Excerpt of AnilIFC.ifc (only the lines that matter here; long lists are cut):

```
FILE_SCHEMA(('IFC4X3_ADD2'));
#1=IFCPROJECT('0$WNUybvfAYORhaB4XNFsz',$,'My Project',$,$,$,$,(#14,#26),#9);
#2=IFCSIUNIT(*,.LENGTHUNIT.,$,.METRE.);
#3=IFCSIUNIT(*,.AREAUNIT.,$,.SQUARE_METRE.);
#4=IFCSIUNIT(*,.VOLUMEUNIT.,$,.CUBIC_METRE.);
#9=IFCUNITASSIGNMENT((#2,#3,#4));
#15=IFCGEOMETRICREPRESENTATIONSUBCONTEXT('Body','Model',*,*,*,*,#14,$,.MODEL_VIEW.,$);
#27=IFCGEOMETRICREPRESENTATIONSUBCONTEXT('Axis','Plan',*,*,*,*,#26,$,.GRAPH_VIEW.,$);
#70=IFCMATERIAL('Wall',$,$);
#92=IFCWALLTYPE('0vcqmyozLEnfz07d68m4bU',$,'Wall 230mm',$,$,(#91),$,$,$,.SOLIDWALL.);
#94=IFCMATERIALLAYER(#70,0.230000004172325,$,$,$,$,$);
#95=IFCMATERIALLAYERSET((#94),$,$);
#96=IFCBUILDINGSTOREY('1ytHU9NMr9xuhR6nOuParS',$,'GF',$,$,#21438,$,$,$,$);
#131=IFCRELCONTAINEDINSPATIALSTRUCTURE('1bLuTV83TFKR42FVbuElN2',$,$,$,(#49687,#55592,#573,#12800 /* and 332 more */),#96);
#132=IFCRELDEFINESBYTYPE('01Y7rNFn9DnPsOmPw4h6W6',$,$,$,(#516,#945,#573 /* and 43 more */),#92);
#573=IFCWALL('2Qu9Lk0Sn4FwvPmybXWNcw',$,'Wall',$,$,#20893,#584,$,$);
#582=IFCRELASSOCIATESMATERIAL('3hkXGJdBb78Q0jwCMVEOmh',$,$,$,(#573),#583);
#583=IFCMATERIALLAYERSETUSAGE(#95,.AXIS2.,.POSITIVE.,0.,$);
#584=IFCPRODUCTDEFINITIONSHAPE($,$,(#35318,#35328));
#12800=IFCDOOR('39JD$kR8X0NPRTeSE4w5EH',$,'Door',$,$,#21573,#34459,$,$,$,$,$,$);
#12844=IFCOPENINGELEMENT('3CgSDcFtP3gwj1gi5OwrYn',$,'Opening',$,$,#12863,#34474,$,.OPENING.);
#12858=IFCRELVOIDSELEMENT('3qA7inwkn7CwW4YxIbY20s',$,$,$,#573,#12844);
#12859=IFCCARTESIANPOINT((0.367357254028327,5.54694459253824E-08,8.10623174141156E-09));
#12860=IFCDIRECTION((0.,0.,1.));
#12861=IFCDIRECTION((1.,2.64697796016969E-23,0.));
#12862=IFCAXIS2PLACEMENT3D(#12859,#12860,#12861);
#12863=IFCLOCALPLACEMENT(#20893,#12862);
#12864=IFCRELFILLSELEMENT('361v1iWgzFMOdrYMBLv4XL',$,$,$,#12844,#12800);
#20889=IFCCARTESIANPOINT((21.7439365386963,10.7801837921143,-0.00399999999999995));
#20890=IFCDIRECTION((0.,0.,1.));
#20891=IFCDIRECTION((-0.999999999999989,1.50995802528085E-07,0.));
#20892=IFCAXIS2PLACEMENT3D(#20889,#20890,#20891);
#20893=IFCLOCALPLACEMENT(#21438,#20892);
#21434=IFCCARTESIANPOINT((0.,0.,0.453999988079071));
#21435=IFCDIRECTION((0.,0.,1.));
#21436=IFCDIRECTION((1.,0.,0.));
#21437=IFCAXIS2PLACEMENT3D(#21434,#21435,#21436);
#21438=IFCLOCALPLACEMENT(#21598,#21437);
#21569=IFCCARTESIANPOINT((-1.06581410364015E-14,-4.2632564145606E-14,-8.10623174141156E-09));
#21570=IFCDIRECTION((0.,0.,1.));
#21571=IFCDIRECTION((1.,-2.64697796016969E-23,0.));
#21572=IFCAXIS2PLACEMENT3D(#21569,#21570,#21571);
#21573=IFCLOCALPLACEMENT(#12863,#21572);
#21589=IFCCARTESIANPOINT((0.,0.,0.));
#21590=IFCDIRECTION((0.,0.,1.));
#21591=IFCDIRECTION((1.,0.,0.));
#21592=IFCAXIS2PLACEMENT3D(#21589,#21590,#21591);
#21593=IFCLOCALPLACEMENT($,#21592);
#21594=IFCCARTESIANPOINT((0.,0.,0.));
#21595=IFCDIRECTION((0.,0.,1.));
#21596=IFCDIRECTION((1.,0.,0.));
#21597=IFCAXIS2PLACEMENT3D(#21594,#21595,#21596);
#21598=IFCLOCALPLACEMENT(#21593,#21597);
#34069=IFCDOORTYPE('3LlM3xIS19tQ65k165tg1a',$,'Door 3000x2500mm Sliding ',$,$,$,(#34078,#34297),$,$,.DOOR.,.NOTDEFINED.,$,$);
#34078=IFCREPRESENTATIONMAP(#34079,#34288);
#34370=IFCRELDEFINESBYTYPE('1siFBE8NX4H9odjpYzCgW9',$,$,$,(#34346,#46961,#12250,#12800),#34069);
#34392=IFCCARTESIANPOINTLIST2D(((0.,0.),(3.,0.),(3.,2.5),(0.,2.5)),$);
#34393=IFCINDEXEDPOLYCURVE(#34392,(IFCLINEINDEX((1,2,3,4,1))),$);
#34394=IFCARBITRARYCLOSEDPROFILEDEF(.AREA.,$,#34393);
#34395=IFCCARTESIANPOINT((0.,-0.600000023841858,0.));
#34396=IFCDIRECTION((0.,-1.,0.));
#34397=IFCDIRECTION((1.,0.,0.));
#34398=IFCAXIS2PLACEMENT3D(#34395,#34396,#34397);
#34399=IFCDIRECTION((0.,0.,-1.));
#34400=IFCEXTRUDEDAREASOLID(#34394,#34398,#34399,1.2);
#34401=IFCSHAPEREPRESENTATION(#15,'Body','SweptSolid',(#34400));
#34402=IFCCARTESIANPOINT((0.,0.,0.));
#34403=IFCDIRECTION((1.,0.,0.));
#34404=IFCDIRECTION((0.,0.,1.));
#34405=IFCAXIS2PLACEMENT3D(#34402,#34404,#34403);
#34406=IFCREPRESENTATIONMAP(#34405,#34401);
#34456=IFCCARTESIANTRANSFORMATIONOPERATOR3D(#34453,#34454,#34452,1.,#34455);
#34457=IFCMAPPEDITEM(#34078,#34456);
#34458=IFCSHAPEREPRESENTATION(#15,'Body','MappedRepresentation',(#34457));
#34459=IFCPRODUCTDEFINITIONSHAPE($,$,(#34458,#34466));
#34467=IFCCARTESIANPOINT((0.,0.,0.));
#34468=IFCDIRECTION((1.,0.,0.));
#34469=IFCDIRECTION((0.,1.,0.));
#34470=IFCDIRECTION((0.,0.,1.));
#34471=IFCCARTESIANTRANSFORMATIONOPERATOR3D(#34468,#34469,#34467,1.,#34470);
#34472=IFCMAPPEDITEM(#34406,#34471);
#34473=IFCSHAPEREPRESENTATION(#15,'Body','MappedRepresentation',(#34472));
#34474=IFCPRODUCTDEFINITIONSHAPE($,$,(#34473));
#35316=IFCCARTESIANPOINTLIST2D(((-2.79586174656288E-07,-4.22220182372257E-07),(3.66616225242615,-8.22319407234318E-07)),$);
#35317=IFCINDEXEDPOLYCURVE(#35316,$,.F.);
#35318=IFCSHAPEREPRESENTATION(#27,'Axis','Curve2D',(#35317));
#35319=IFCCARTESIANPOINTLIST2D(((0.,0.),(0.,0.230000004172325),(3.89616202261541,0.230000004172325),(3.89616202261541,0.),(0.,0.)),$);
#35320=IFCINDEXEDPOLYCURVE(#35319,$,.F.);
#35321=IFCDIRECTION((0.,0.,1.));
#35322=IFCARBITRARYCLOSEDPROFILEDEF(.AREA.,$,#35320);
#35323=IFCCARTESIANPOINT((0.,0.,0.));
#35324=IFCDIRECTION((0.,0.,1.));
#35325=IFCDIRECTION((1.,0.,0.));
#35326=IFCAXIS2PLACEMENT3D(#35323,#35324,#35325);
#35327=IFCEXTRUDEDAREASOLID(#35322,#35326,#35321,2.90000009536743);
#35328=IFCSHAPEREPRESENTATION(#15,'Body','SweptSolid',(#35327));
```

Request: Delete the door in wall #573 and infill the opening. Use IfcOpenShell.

```python
import ifcopenshell
import ifcopenshell.api.feature
import ifcopenshell.api.root
import ifcopenshell.geom
import ifcopenshell.util.shape

model = ifcopenshell.open("AnilIFC.ifc")
settings = ifcopenshell.geom.settings()


def volume(element):
    """Net volume in cubic metres, openings subtracted."""
    shape = ifcopenshell.geom.create_shape(settings, element)
    return ifcopenshell.util.shape.get_volume(shape.geometry)


door = model.by_guid("39JD$kR8X0NPRTeSE4w5EH")
opening = door.FillsVoids[0].RelatingOpeningElement
wall = opening.VoidsElements[0].RelatingBuildingElement
before = volume(wall)

ifcopenshell.api.root.remove_product(model, product=door)
ifcopenshell.api.feature.remove_feature(model, feature=opening)

after = volume(wall)

print(f"wall volume {before:.3f} -> {after:.3f} m3")

model.write("AnilIFC_rev.ifc")
```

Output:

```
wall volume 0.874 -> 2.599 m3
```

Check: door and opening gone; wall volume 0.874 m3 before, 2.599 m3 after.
